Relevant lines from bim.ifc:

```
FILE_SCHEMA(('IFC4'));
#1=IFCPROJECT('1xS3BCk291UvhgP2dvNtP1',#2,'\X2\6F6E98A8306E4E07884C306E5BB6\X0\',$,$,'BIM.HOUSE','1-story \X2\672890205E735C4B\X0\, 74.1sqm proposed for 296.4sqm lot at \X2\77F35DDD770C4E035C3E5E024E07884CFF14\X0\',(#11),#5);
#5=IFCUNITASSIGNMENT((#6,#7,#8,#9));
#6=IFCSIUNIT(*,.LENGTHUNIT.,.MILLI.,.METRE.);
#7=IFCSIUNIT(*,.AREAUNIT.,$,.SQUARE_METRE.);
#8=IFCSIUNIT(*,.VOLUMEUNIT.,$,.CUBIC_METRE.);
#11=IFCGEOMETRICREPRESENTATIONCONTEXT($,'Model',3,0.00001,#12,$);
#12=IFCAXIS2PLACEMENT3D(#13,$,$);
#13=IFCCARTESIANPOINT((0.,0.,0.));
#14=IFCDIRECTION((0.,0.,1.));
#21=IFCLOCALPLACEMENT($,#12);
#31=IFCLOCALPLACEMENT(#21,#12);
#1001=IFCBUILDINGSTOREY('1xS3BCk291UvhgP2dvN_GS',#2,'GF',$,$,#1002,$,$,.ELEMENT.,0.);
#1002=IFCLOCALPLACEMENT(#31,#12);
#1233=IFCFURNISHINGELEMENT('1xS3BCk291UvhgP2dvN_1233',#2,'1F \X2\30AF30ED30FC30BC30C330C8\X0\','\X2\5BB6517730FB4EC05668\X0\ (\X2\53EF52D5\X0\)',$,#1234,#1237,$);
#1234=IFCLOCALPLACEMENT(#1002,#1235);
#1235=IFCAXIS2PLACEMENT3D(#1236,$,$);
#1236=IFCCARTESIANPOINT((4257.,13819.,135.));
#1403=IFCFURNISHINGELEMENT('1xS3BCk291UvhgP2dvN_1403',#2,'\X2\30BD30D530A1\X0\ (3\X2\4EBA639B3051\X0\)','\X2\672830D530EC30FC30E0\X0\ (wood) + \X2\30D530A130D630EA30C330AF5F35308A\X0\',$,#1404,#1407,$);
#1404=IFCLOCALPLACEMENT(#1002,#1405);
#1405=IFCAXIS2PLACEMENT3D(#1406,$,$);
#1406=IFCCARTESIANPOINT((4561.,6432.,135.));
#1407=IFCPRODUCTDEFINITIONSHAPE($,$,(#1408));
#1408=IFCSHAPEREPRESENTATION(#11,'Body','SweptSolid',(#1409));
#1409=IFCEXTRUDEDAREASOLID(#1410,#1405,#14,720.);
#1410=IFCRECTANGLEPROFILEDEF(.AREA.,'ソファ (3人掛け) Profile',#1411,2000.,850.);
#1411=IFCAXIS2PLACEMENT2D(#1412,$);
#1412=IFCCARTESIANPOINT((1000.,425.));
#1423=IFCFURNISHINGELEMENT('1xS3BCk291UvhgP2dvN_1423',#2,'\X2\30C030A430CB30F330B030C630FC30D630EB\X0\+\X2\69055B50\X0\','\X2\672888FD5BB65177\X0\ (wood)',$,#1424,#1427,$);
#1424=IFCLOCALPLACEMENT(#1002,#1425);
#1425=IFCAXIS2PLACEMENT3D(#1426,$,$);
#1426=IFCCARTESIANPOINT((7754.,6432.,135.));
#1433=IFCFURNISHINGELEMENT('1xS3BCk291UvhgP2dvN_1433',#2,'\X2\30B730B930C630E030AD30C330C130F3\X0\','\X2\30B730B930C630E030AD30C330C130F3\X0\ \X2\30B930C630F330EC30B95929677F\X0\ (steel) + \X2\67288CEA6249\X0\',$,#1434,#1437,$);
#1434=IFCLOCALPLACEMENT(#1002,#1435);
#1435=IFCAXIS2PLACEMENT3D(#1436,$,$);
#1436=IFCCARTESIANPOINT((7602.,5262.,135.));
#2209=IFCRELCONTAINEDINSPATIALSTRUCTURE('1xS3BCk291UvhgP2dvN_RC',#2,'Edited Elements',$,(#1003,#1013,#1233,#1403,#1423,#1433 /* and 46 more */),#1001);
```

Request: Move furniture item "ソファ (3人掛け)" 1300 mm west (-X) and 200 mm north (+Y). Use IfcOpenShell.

```python
import ifcopenshell
import ifcopenshell.api.geometry
import ifcopenshell.util.placement
import ifcopenshell.util.unit

model = ifcopenshell.open("bim.ifc")
unit_scale = ifcopenshell.util.unit.calculate_unit_scale(model)

item = model.by_guid("1xS3BCk291UvhgP2dvN_1403")
matrix = ifcopenshell.util.placement.get_local_placement(item.ObjectPlacement)
matrix[0, 3] -= 1.3 / unit_scale
matrix[1, 3] += 0.2 / unit_scale
ifcopenshell.api.geometry.edit_object_placement(model, product=item, matrix=matrix, is_si=False)

print(ifcopenshell.util.placement.get_local_placement(item.ObjectPlacement).round(3) + 0.0)

model.write("bim_rev.ifc")
```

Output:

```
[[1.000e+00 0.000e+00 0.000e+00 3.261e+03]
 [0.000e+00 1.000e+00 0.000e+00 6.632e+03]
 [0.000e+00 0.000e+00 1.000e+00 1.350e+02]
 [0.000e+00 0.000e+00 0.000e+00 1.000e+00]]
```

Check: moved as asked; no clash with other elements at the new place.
